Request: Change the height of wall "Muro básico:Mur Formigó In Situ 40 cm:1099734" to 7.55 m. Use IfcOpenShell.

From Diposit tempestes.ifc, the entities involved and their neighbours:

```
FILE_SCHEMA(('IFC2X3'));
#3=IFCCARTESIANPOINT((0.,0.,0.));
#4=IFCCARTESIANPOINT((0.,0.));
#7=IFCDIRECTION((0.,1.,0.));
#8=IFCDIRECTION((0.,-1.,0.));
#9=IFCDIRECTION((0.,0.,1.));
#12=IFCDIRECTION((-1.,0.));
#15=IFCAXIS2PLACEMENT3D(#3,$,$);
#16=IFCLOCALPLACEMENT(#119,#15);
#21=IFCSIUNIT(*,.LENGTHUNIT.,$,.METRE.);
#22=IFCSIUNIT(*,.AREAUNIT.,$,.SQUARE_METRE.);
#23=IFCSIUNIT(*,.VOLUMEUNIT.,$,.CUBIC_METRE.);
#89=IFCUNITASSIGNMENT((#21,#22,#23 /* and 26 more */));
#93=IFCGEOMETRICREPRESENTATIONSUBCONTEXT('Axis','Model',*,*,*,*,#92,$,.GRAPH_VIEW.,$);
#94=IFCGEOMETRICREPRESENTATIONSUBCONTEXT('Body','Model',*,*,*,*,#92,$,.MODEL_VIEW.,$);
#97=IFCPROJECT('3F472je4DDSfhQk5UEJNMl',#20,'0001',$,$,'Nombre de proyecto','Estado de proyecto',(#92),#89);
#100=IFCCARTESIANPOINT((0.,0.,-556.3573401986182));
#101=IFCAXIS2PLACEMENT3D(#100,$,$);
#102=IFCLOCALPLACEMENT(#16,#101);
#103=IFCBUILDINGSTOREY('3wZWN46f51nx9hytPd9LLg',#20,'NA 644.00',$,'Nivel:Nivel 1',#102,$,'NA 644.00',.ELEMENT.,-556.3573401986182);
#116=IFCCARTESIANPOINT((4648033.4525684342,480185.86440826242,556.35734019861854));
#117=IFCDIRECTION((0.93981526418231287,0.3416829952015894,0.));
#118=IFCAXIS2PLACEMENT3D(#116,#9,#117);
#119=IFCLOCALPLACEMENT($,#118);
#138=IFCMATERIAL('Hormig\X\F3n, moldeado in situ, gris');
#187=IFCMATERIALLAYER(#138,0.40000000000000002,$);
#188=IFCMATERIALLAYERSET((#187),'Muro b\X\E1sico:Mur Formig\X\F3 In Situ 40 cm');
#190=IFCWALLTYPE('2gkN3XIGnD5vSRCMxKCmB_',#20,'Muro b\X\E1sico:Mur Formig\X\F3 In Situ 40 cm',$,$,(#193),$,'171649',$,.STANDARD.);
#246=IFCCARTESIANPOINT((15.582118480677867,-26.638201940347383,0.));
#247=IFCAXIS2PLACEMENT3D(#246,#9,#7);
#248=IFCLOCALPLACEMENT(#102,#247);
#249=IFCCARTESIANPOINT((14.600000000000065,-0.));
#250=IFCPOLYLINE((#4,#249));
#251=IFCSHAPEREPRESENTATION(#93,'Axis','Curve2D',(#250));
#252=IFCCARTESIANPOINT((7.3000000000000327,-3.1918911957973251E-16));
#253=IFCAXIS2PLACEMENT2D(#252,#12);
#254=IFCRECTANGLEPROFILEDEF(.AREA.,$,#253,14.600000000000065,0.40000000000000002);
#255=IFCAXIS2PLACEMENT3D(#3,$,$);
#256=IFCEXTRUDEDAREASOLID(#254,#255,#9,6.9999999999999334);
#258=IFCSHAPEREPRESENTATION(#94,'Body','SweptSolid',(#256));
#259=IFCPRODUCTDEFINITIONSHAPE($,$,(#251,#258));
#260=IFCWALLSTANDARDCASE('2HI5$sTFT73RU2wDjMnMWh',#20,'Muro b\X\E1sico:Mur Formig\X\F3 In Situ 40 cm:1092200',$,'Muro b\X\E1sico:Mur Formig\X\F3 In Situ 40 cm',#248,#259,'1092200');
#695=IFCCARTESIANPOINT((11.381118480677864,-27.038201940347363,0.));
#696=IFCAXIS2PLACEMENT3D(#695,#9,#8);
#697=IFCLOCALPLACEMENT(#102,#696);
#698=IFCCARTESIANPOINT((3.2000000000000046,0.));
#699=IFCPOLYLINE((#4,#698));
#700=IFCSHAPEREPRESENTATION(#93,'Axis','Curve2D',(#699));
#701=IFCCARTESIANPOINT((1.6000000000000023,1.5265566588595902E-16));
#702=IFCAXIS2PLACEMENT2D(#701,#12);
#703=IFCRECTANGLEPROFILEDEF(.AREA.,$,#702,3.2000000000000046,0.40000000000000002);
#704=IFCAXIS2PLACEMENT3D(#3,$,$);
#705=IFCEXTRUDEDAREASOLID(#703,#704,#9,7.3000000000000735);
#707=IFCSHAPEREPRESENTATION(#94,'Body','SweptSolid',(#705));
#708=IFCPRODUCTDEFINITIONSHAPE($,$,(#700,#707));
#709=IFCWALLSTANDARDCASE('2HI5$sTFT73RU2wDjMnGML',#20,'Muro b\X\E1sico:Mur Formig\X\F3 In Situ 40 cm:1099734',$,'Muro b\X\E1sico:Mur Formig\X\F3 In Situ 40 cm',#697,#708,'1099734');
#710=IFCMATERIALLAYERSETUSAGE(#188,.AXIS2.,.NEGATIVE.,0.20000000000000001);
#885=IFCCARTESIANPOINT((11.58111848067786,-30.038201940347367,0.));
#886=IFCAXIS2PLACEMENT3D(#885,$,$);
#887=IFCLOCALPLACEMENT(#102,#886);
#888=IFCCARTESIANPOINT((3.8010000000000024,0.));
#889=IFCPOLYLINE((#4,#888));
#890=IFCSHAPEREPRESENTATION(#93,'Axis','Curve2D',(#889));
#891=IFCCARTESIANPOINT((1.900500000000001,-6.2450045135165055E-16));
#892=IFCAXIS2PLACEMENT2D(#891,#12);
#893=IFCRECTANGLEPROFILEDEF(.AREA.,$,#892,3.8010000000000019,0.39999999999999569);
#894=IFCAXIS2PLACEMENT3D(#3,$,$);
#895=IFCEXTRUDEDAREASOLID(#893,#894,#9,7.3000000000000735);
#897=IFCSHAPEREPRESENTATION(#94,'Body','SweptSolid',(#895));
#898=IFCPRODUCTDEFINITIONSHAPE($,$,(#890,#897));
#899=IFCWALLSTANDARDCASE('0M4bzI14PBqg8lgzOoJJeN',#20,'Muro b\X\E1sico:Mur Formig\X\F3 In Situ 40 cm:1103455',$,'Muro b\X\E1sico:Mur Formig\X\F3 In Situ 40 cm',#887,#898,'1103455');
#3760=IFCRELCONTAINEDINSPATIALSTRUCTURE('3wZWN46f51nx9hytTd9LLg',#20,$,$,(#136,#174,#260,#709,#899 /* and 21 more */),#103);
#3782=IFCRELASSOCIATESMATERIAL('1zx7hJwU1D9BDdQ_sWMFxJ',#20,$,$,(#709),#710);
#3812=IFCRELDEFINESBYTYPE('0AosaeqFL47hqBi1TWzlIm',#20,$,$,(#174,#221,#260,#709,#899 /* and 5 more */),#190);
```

```python
import ifcopenshell
import ifcopenshell.geom
import ifcopenshell.util.representation
import ifcopenshell.util.shape
import ifcopenshell.util.unit

model = ifcopenshell.open("Diposit tempestes.ifc")
unit_scale = ifcopenshell.util.unit.calculate_unit_scale(model)
settings = ifcopenshell.geom.settings()


def volume(element):
    """Net volume in cubic metres, openings subtracted."""
    shape = ifcopenshell.geom.create_shape(settings, element)
    return ifcopenshell.util.shape.get_volume(shape.geometry)


wall = model.by_guid("2HI5$sTFT73RU2wDjMnGML")
before = volume(wall)

body = ifcopenshell.util.representation.get_representation(wall, "Model", "Body")
solid = body.Items[0]
old_height = solid.Depth
solid.Depth = 7.55 / unit_scale
after = volume(wall)

print(f"height {old_height:g} -> {solid.Depth:g}, volume {before:.3f} -> {after:.3f} m3")

model.write("Diposit tempestes_v2.ifc")
```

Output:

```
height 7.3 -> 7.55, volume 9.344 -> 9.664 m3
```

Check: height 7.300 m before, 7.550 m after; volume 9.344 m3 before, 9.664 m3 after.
